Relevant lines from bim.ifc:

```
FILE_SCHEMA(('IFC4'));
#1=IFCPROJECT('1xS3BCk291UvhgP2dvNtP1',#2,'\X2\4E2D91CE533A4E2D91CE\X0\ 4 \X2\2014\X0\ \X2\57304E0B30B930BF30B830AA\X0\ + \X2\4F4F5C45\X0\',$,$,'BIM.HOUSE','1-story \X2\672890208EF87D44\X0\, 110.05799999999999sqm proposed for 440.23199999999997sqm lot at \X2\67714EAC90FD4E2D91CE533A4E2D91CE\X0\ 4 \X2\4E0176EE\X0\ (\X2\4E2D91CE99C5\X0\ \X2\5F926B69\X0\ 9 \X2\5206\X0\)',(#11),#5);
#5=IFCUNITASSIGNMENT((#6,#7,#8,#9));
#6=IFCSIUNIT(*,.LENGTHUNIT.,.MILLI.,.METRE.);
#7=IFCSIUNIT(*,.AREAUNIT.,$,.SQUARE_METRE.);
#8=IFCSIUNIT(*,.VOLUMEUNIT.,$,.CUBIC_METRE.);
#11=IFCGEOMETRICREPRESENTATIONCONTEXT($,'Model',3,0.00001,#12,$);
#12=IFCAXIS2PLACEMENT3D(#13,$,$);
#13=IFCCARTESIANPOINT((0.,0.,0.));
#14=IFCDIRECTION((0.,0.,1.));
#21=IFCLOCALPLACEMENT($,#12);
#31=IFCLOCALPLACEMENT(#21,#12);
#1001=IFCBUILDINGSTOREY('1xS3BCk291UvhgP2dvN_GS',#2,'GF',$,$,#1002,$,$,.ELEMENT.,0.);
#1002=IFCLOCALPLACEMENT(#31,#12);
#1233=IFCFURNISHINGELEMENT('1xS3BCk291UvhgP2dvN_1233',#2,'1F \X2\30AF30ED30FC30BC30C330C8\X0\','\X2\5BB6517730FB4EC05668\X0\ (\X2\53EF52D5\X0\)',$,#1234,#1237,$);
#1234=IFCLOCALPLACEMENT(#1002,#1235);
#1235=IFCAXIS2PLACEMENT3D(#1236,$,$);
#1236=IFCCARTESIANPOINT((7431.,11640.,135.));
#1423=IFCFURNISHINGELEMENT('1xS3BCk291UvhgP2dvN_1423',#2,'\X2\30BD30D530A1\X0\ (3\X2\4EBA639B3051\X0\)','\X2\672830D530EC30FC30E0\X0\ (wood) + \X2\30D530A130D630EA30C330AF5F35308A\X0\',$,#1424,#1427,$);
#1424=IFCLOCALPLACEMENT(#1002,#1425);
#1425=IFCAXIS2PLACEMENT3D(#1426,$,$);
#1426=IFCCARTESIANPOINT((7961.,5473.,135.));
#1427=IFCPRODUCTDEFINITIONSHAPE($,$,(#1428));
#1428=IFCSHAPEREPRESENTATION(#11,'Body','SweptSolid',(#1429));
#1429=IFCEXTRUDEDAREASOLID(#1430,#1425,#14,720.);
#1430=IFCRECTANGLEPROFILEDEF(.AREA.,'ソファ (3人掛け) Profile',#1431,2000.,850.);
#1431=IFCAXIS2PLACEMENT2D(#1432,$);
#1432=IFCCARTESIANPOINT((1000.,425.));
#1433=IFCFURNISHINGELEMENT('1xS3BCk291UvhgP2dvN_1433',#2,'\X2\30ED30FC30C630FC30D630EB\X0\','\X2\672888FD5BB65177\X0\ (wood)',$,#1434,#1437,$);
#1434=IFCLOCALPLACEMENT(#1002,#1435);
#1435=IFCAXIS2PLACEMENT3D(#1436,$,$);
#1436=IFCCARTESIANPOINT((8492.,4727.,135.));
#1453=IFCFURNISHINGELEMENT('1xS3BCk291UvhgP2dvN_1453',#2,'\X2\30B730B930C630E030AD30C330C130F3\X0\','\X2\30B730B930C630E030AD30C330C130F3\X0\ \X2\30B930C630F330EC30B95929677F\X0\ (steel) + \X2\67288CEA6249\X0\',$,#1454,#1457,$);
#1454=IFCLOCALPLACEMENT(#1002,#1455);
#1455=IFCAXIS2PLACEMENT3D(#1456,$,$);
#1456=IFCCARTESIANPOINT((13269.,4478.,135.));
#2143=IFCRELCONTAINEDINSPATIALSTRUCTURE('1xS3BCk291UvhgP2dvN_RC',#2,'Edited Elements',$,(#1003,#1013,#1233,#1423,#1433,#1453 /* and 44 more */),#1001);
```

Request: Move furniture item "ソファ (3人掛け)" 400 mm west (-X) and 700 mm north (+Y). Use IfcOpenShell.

```python
import ifcopenshell
import ifcopenshell.api.geometry
import ifcopenshell.util.placement

model = ifcopenshell.open("bim.ifc")

item = model.by_id(1423)
matrix = ifcopenshell.util.placement.get_local_placement(item.ObjectPlacement)
matrix[0, 3] -= 400.0
matrix[1, 3] += 700.0
ifcopenshell.api.geometry.edit_object_placement(model, product=item, matrix=matrix, is_si=False)

print(ifcopenshell.util.placement.get_local_placement(item.ObjectPlacement).round(3) + 0.0)

model.write("bim_edited.ifc")
```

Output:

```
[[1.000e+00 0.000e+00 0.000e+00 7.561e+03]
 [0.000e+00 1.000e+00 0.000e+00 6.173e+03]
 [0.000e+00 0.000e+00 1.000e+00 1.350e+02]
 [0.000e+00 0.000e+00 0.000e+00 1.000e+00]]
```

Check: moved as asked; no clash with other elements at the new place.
